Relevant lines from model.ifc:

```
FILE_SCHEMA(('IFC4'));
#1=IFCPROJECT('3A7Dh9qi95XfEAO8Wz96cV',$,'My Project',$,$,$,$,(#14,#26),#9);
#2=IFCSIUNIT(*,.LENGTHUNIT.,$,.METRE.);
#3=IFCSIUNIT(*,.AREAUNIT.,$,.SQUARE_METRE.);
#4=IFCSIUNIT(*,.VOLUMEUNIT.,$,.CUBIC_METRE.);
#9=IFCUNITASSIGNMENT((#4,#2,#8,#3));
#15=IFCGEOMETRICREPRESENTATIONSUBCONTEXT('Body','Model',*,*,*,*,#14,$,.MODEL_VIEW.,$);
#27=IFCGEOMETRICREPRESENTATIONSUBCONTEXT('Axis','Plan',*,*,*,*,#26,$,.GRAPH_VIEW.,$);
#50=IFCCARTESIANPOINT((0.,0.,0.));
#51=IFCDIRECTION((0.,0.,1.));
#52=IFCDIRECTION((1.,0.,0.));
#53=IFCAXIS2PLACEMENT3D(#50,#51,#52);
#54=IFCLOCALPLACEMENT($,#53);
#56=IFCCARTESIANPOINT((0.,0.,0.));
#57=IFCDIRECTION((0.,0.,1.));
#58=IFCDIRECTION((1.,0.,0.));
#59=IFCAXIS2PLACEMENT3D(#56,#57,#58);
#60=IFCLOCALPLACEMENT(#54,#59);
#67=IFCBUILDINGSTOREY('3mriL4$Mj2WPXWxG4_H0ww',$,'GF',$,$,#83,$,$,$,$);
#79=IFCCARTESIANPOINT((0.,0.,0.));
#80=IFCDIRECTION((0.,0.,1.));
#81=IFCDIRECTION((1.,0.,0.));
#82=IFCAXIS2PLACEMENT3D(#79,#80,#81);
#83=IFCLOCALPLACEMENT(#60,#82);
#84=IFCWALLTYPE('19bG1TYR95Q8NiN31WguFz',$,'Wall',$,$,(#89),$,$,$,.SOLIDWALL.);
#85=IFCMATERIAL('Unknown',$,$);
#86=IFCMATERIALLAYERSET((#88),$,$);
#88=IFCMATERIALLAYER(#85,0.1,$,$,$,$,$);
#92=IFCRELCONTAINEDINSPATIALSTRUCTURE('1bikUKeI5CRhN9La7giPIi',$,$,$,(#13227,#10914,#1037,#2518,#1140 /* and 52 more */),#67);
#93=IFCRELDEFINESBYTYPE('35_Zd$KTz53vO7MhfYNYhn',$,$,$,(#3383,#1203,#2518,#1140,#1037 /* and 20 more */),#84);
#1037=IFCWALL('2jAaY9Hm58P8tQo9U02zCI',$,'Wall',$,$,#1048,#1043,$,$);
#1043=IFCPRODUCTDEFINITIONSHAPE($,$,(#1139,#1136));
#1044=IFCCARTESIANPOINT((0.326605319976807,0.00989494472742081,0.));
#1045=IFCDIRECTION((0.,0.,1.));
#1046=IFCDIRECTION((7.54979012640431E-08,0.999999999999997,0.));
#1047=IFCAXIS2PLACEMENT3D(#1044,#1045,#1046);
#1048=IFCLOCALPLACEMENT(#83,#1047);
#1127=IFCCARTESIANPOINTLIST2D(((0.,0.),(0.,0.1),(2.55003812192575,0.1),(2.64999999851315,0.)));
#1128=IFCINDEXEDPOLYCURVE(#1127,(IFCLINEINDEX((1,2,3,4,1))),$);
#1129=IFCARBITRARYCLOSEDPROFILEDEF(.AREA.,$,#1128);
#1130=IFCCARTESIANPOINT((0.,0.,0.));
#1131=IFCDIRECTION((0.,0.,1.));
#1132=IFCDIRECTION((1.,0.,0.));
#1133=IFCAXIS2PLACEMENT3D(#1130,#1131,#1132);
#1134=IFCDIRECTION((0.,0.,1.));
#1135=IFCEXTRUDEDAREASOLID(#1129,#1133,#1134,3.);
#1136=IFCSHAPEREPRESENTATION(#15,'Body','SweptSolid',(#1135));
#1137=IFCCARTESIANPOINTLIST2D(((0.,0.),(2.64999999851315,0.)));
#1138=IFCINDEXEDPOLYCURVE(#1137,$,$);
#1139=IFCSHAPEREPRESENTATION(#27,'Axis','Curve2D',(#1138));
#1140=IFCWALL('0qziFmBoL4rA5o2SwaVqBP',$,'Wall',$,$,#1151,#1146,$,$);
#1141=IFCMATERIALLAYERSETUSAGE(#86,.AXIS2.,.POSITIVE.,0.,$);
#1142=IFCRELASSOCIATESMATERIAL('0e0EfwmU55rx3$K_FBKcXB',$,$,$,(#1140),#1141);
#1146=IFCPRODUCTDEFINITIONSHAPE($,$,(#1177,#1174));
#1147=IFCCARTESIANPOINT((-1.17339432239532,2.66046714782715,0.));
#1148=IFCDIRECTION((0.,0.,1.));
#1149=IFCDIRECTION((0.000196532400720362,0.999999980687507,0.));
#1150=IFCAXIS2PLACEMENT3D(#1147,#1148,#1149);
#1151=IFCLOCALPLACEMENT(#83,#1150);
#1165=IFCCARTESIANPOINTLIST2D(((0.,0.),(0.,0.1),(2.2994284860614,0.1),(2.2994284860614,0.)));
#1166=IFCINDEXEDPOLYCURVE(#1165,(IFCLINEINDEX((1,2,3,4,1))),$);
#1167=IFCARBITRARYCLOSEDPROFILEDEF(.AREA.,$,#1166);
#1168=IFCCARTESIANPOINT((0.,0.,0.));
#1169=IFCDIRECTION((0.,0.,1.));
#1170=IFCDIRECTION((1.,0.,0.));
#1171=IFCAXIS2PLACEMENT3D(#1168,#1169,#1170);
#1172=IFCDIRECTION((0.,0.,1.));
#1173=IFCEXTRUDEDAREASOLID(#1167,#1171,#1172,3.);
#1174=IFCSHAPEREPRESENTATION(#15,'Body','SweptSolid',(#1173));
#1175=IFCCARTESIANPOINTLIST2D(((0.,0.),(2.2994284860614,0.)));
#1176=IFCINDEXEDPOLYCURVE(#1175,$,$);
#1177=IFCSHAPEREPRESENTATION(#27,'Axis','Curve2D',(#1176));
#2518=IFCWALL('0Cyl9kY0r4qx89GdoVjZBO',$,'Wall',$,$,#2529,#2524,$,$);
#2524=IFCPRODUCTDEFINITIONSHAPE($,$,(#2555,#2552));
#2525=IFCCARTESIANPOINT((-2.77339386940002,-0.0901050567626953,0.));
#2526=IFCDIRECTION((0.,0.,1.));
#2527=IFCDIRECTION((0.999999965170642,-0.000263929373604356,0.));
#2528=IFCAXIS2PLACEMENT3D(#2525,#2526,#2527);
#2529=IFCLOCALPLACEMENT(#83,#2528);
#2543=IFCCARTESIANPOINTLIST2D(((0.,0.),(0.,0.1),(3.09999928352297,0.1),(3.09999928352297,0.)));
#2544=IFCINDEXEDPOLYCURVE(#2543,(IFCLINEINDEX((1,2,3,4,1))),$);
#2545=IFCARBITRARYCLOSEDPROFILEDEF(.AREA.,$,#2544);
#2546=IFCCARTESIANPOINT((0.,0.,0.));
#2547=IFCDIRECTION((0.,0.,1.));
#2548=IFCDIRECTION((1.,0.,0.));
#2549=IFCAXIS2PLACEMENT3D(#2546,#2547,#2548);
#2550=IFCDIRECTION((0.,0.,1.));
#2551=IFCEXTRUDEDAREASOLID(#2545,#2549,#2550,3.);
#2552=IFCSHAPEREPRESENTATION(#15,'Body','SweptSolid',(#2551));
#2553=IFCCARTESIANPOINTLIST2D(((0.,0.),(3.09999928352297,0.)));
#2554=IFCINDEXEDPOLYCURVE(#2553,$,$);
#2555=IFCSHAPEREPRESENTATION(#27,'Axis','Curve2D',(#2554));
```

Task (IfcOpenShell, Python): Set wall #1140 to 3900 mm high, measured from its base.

```python
import ifcopenshell
import ifcopenshell.geom
import ifcopenshell.util.representation
import ifcopenshell.util.shape
import ifcopenshell.util.unit

model = ifcopenshell.open("model.ifc")
unit_scale = ifcopenshell.util.unit.calculate_unit_scale(model)
settings = ifcopenshell.geom.settings()


def volume(element):
    """Net volume in cubic metres, openings subtracted."""
    shape = ifcopenshell.geom.create_shape(settings, element)
    return ifcopenshell.util.shape.get_volume(shape.geometry)


wall = model.by_guid("0qziFmBoL4rA5o2SwaVqBP")
before = volume(wall)

body = ifcopenshell.util.representation.get_representation(wall, "Model", "Body")
solid = body.Items[0]
old_height = solid.Depth
solid.Depth = 3.9 / unit_scale
after = volume(wall)

print(f"height {old_height:g} -> {solid.Depth:g}, volume {before:.3f} -> {after:.3f} m3")

model.write("model_v2.ifc")
```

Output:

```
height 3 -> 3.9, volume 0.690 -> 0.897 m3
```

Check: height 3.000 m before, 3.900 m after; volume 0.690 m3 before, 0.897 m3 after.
